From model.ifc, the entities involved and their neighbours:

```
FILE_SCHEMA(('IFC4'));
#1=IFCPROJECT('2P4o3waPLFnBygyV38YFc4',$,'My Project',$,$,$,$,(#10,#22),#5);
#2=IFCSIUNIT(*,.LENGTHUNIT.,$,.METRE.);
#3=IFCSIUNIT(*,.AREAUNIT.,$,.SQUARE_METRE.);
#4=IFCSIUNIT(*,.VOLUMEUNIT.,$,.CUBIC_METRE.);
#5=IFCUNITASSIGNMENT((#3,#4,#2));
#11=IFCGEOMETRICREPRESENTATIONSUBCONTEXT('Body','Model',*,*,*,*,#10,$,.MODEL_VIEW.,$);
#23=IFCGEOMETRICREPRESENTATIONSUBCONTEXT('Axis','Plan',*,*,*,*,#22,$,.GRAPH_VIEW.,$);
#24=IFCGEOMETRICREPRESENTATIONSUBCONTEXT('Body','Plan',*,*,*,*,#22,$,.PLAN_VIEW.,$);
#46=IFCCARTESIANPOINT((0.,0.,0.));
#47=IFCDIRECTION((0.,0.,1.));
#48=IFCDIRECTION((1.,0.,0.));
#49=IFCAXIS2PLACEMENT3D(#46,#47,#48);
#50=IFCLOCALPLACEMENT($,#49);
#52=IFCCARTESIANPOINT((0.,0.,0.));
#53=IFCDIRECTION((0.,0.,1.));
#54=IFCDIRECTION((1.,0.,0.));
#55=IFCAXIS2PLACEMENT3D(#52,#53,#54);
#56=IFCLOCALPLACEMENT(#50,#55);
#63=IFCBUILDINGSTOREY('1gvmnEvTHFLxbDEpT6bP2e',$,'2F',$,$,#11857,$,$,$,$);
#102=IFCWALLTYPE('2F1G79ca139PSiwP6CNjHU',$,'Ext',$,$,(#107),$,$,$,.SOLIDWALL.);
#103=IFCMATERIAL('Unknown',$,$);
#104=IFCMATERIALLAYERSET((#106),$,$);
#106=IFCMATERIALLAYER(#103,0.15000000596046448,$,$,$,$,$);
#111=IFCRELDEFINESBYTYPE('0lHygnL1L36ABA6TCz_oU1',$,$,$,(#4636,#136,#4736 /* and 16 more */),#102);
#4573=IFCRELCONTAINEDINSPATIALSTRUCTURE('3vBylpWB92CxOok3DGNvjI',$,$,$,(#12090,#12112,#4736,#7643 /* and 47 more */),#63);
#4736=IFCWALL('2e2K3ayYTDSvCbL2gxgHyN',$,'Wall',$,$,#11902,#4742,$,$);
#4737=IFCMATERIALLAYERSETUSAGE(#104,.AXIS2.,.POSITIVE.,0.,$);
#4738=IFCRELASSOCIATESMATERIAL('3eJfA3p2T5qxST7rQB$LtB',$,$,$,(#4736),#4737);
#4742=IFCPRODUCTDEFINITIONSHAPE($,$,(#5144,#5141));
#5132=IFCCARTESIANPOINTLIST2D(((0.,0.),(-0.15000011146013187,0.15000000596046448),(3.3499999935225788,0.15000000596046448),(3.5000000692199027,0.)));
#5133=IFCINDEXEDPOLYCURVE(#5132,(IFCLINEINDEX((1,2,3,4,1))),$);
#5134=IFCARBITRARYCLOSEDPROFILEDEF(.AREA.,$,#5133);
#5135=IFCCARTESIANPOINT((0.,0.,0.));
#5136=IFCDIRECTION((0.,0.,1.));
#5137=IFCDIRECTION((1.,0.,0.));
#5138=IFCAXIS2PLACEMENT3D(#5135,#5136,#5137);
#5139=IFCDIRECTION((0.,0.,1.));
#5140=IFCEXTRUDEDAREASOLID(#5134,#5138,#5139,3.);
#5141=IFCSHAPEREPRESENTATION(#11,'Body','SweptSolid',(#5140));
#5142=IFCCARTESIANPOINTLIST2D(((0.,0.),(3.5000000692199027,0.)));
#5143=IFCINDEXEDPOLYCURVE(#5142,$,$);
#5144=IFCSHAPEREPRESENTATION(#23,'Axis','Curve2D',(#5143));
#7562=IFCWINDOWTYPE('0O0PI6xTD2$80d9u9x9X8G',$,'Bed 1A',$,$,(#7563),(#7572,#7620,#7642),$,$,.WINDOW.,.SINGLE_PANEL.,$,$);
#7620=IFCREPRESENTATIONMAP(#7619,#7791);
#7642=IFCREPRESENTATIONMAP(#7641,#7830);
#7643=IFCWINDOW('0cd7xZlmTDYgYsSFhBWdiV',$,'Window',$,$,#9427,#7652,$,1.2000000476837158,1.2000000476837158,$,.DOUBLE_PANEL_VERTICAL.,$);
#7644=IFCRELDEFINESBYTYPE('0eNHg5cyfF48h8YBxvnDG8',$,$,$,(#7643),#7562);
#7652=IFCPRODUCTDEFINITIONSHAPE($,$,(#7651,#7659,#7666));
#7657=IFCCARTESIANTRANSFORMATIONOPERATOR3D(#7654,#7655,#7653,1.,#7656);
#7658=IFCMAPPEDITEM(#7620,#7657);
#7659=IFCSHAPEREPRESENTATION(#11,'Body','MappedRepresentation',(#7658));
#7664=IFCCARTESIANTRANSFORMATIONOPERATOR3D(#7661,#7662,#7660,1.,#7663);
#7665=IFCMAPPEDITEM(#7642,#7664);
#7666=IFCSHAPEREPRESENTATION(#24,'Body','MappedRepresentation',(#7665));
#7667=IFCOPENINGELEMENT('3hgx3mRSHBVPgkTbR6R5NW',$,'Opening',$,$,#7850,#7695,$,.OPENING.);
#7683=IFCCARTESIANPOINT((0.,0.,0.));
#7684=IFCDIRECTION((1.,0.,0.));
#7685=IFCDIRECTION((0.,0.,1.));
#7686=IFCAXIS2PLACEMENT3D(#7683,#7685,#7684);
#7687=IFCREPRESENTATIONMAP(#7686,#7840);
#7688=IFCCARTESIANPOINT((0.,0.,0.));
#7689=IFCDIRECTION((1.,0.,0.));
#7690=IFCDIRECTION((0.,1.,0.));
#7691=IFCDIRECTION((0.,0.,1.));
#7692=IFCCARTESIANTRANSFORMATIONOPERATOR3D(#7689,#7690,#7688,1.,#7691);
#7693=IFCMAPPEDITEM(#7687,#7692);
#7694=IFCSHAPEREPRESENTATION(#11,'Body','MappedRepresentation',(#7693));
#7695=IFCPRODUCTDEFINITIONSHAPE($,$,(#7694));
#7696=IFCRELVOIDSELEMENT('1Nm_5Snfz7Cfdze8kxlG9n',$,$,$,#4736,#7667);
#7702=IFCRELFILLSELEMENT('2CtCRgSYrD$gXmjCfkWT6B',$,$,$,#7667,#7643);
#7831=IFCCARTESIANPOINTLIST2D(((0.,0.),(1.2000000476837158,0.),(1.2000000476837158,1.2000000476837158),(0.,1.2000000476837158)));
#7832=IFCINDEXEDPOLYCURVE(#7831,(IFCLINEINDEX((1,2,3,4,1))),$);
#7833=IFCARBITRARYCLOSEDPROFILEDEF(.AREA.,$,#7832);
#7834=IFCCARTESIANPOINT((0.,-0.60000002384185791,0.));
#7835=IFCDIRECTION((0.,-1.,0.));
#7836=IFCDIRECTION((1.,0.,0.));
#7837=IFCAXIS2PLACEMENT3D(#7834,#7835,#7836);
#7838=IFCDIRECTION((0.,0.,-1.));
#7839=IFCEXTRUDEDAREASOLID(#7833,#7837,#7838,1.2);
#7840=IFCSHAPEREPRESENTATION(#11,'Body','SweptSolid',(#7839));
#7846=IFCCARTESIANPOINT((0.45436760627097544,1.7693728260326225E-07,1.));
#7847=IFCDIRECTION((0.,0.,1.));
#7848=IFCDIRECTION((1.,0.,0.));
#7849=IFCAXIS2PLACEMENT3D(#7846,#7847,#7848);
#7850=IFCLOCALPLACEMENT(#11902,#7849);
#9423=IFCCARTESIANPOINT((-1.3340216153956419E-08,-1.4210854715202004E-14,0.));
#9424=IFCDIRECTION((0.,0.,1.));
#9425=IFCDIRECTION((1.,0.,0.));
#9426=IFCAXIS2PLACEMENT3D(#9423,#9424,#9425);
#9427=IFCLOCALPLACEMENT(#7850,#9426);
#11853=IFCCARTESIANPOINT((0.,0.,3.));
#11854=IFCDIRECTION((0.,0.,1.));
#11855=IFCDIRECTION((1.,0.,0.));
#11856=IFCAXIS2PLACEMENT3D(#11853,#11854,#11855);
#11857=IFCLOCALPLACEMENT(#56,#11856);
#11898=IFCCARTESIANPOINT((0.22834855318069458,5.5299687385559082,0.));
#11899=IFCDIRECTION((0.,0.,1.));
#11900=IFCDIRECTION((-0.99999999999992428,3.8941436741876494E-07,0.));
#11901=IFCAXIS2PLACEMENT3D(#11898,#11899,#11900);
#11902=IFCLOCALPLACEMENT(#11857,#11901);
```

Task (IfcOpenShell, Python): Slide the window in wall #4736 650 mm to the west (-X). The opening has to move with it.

```python
import ifcopenshell
import ifcopenshell.api.geometry
import ifcopenshell.util.placement
import ifcopenshell.util.unit

model = ifcopenshell.open("model.ifc")
unit_scale = ifcopenshell.util.unit.calculate_unit_scale(model)

window = model.by_guid("0cd7xZlmTDYgYsSFhBWdiV")
opening = window.FillsVoids[0].RelatingOpeningElement
wall = opening.VoidsElements[0].RelatingBuildingElement

wall_matrix = ifcopenshell.util.placement.get_local_placement(wall.ObjectPlacement)
shift = wall_matrix[:3, 0] * 0.65 / unit_scale
before = ifcopenshell.util.placement.get_local_placement(window.ObjectPlacement)[:3, 3].copy()

# The window is placed relative to its opening, so it follows when the opening moves.
matrix = ifcopenshell.util.placement.get_local_placement(opening.ObjectPlacement)
matrix[:3, 3] += shift
ifcopenshell.api.geometry.edit_object_placement(
    model, product=opening, matrix=matrix, is_si=False, should_transform_children=True
)

after = ifcopenshell.util.placement.get_local_placement(window.ObjectPlacement)[:3, 3]
print("window moved by", (after - before).round(3) + 0.0)

model.write("model-out.ifc")
```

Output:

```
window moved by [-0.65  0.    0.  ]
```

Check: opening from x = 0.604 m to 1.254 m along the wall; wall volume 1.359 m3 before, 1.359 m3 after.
